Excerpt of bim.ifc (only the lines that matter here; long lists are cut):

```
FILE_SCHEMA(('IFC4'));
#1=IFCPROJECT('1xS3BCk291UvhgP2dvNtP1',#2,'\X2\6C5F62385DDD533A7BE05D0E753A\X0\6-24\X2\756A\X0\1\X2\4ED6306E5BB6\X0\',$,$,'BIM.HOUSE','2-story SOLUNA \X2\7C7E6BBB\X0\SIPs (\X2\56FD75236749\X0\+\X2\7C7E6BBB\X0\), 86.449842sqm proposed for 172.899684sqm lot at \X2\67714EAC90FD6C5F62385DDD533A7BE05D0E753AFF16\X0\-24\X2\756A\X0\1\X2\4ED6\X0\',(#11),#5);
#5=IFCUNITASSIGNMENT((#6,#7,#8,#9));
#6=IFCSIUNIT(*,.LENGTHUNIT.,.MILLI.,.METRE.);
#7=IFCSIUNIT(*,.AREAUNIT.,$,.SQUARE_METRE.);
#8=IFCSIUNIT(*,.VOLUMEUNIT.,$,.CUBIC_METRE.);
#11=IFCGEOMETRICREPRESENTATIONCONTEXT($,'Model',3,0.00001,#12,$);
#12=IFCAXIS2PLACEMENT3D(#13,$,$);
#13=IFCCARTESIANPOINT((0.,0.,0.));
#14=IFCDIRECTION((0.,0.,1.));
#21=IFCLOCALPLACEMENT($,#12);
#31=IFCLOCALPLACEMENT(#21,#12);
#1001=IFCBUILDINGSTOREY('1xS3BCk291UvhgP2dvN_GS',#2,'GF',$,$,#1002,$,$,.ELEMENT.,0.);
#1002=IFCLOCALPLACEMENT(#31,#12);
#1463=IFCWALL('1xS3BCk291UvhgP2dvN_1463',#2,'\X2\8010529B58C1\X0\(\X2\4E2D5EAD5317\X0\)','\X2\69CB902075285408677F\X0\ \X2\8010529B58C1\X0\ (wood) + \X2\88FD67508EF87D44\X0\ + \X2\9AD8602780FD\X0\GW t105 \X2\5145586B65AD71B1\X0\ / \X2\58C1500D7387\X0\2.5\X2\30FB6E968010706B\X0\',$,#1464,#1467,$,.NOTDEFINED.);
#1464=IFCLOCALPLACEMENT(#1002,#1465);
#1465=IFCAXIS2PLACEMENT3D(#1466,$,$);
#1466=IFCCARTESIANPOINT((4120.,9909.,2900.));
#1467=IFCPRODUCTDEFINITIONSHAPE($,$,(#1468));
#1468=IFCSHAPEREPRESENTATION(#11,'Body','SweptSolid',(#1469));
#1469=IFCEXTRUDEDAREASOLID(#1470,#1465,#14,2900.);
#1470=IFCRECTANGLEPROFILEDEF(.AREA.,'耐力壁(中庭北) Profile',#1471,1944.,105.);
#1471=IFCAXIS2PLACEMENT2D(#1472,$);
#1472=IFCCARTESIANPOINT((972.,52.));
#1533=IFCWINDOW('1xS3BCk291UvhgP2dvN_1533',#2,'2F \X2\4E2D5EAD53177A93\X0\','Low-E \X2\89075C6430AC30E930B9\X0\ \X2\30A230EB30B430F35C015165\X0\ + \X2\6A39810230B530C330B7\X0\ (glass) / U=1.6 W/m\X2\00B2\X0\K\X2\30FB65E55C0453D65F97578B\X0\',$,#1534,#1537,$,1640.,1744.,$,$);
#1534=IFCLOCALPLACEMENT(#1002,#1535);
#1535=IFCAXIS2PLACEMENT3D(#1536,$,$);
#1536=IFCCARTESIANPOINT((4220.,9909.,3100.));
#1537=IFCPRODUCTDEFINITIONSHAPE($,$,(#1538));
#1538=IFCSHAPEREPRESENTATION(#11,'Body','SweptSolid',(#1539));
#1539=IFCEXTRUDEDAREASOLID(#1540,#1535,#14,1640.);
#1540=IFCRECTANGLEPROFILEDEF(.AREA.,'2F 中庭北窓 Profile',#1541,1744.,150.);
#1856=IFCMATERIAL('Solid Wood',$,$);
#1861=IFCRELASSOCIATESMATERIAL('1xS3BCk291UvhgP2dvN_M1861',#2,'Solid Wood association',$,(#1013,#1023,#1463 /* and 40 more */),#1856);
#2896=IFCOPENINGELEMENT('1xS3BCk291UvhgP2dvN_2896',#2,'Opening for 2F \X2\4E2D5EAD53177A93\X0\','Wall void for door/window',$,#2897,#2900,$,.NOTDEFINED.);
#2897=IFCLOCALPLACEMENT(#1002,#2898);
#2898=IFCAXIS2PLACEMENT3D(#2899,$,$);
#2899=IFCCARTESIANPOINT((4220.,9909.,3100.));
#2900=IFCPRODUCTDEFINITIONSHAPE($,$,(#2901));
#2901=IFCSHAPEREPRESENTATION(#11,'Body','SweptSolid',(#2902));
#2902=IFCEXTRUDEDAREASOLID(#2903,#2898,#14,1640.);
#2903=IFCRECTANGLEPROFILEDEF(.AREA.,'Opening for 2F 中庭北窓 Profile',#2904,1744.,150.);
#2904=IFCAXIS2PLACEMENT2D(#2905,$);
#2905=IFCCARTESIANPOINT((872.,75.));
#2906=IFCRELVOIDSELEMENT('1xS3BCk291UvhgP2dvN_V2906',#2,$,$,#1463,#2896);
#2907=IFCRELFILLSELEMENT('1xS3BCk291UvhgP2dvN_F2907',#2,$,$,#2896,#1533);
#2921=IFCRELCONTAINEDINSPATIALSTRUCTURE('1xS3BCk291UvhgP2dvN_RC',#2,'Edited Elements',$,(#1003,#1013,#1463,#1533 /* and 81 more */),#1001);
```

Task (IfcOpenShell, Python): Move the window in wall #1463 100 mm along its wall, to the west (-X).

```python
import ifcopenshell
import ifcopenshell.api.geometry
import ifcopenshell.util.placement

model = ifcopenshell.open("bim.ifc")

window = model.by_id(1533)
opening = window.FillsVoids[0].RelatingOpeningElement
wall = opening.VoidsElements[0].RelatingBuildingElement

wall_matrix = ifcopenshell.util.placement.get_local_placement(wall.ObjectPlacement)
shift = wall_matrix[:3, 0] * -100.0
before = ifcopenshell.util.placement.get_local_placement(window.ObjectPlacement)[:3, 3].copy()

# The window is not placed relative to its opening, so move both.
for product in (opening, window):
    matrix = ifcopenshell.util.placement.get_local_placement(product.ObjectPlacement)
    matrix[:3, 3] += shift
    ifcopenshell.api.geometry.edit_object_placement(model, product=product, matrix=matrix, is_si=False)

after = ifcopenshell.util.placement.get_local_placement(window.ObjectPlacement)[:3, 3]
print("window moved by", (after - before).round(3) + 0.0)

model.write("bim_updated.ifc")
```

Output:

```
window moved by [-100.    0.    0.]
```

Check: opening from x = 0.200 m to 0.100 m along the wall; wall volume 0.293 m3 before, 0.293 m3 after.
